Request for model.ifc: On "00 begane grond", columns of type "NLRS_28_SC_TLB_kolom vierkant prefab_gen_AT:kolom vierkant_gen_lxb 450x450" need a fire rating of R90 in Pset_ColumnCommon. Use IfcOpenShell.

First a look at what the model holds.

```python
import ifcopenshell
import ifcopenshell.util.element

model = ifcopenshell.open("model.ifc")
print(model.schema)
storey = next(s for s in model.by_type("IfcBuildingStorey") if s.Name == "00 begane grond")
columns = [e for e in ifcopenshell.util.element.get_decomposition(storey) if e.is_a("IfcColumn")]
seen = {}
for e in columns:
    element_type = ifcopenshell.util.element.get_type(e)
    key = (element_type.Name if element_type != e and element_type else None, ifcopenshell.util.element.get_pset(e, "Pset_ColumnCommon", "FireRating"))
    seen[key] = seen.get(key, 0) + 1
for (name, value), count in sorted(seen.items(), key=str):
    print(count, "x", name, "|", value)
```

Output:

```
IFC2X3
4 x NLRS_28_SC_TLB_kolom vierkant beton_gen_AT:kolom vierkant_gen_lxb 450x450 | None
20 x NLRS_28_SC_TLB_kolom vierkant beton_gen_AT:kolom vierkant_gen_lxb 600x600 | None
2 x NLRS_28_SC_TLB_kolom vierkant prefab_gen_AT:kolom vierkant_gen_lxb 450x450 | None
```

```python
import ifcopenshell
import ifcopenshell.api.pset
import ifcopenshell.util.element

model = ifcopenshell.open("model.ifc")

storey = next(s for s in model.by_type("IfcBuildingStorey") if s.Name == "00 begane grond")
columns = [e for e in ifcopenshell.util.element.get_decomposition(storey) if e.is_a("IfcColumn")]

count = 0
for e in columns:
    element_type = ifcopenshell.util.element.get_type(e)
    if element_type in (None, e) or element_type.Name != "NLRS_28_SC_TLB_kolom vierkant prefab_gen_AT:kolom vierkant_gen_lxb 450x450":
        continue
    found = ifcopenshell.util.element.get_pset(e, "Pset_ColumnCommon", should_inherit=False)
    if found:
        pset = model.by_id(found["id"])
        if len(ifcopenshell.util.element.get_elements_by_pset(pset)) > 1:
            pset = ifcopenshell.api.pset.unshare_pset(model, products=[e], pset=pset)[0]
    else:
        pset = ifcopenshell.api.pset.add_pset(model, product=e, name="Pset_ColumnCommon")
    ifcopenshell.api.pset.edit_pset(model, pset=pset, properties={"FireRating": "R90"})
    count += 1

print(count, "columns updated")

model.write("model_v2.ifc")
```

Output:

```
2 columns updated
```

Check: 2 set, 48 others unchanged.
